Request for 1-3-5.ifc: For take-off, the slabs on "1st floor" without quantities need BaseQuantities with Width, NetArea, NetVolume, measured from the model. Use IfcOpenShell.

First a look at what the model holds.

```python
import ifcopenshell
import ifcopenshell.util.element
import ifcopenshell.util.unit

model = ifcopenshell.open("1-3-5.ifc")
print(model.schema)
for unit_type in ("LENGTHUNIT", "AREAUNIT", "VOLUMEUNIT"):
    print(unit_type, ifcopenshell.util.unit.calculate_unit_scale(model, unit_type))
storey = next(s for s in model.by_type("IfcBuildingStorey") if s.Name == "1st floor")
slabs = [e for e in ifcopenshell.util.element.get_decomposition(storey) if e.is_a("IfcSlab")]
for e in sorted(slabs, key=lambda e: e.id()):
    print(e.id(), e.is_a(), e.Name, list(ifcopenshell.util.element.get_psets(e, qtos_only=True)), sep=" | ")
```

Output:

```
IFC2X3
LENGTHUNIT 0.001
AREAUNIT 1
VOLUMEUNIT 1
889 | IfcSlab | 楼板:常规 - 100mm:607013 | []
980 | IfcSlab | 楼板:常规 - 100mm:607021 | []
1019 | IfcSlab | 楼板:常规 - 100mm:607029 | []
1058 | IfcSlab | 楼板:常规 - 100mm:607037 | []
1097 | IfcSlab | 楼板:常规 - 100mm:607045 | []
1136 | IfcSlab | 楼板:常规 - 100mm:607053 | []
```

```python
import ifcopenshell
import ifcopenshell.api.pset
import ifcopenshell.geom
import ifcopenshell.util.element
import ifcopenshell.util.shape
import ifcopenshell.util.unit

model = ifcopenshell.open("1-3-5.ifc")
unit_scale = ifcopenshell.util.unit.calculate_unit_scale(model)
area_scale = ifcopenshell.util.unit.calculate_unit_scale(model, "AREAUNIT")
volume_scale = ifcopenshell.util.unit.calculate_unit_scale(model, "VOLUMEUNIT")
settings = ifcopenshell.geom.settings()

storey = next(s for s in model.by_type("IfcBuildingStorey") if s.Name == "1st floor")
slabs = [e for e in ifcopenshell.util.element.get_decomposition(storey) if e.is_a("IfcSlab")]

for e in sorted(slabs, key=lambda e: e.id()):
    if ifcopenshell.util.element.get_psets(e, qtos_only=True, should_inherit=False):
        continue
    # Geometry comes back in metres, in the element's own axes.
    shape = ifcopenshell.geom.create_shape(settings, e)
    values = {
        "Width": ifcopenshell.util.shape.get_z(shape.geometry) / unit_scale,
        "NetArea": ifcopenshell.util.shape.get_footprint_area(shape.geometry) / area_scale,
        "NetVolume": ifcopenshell.util.shape.get_volume(shape.geometry) / volume_scale,
    }
    qto = ifcopenshell.api.pset.add_qto(model, product=e, name="BaseQuantities")
    ifcopenshell.api.pset.edit_qto(model, qto=qto, properties=values)
    print(e.id(), {k: round(v, 3) for k, v in values.items()})

model.write("1-3-5_rev.ifc")
```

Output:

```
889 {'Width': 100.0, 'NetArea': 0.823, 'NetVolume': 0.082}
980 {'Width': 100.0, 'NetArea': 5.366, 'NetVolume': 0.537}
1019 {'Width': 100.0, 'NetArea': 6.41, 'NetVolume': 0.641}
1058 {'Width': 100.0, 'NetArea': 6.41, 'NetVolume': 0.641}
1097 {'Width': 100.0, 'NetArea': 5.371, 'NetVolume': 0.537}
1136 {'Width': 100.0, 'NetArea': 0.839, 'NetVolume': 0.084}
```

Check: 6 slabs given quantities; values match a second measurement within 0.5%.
